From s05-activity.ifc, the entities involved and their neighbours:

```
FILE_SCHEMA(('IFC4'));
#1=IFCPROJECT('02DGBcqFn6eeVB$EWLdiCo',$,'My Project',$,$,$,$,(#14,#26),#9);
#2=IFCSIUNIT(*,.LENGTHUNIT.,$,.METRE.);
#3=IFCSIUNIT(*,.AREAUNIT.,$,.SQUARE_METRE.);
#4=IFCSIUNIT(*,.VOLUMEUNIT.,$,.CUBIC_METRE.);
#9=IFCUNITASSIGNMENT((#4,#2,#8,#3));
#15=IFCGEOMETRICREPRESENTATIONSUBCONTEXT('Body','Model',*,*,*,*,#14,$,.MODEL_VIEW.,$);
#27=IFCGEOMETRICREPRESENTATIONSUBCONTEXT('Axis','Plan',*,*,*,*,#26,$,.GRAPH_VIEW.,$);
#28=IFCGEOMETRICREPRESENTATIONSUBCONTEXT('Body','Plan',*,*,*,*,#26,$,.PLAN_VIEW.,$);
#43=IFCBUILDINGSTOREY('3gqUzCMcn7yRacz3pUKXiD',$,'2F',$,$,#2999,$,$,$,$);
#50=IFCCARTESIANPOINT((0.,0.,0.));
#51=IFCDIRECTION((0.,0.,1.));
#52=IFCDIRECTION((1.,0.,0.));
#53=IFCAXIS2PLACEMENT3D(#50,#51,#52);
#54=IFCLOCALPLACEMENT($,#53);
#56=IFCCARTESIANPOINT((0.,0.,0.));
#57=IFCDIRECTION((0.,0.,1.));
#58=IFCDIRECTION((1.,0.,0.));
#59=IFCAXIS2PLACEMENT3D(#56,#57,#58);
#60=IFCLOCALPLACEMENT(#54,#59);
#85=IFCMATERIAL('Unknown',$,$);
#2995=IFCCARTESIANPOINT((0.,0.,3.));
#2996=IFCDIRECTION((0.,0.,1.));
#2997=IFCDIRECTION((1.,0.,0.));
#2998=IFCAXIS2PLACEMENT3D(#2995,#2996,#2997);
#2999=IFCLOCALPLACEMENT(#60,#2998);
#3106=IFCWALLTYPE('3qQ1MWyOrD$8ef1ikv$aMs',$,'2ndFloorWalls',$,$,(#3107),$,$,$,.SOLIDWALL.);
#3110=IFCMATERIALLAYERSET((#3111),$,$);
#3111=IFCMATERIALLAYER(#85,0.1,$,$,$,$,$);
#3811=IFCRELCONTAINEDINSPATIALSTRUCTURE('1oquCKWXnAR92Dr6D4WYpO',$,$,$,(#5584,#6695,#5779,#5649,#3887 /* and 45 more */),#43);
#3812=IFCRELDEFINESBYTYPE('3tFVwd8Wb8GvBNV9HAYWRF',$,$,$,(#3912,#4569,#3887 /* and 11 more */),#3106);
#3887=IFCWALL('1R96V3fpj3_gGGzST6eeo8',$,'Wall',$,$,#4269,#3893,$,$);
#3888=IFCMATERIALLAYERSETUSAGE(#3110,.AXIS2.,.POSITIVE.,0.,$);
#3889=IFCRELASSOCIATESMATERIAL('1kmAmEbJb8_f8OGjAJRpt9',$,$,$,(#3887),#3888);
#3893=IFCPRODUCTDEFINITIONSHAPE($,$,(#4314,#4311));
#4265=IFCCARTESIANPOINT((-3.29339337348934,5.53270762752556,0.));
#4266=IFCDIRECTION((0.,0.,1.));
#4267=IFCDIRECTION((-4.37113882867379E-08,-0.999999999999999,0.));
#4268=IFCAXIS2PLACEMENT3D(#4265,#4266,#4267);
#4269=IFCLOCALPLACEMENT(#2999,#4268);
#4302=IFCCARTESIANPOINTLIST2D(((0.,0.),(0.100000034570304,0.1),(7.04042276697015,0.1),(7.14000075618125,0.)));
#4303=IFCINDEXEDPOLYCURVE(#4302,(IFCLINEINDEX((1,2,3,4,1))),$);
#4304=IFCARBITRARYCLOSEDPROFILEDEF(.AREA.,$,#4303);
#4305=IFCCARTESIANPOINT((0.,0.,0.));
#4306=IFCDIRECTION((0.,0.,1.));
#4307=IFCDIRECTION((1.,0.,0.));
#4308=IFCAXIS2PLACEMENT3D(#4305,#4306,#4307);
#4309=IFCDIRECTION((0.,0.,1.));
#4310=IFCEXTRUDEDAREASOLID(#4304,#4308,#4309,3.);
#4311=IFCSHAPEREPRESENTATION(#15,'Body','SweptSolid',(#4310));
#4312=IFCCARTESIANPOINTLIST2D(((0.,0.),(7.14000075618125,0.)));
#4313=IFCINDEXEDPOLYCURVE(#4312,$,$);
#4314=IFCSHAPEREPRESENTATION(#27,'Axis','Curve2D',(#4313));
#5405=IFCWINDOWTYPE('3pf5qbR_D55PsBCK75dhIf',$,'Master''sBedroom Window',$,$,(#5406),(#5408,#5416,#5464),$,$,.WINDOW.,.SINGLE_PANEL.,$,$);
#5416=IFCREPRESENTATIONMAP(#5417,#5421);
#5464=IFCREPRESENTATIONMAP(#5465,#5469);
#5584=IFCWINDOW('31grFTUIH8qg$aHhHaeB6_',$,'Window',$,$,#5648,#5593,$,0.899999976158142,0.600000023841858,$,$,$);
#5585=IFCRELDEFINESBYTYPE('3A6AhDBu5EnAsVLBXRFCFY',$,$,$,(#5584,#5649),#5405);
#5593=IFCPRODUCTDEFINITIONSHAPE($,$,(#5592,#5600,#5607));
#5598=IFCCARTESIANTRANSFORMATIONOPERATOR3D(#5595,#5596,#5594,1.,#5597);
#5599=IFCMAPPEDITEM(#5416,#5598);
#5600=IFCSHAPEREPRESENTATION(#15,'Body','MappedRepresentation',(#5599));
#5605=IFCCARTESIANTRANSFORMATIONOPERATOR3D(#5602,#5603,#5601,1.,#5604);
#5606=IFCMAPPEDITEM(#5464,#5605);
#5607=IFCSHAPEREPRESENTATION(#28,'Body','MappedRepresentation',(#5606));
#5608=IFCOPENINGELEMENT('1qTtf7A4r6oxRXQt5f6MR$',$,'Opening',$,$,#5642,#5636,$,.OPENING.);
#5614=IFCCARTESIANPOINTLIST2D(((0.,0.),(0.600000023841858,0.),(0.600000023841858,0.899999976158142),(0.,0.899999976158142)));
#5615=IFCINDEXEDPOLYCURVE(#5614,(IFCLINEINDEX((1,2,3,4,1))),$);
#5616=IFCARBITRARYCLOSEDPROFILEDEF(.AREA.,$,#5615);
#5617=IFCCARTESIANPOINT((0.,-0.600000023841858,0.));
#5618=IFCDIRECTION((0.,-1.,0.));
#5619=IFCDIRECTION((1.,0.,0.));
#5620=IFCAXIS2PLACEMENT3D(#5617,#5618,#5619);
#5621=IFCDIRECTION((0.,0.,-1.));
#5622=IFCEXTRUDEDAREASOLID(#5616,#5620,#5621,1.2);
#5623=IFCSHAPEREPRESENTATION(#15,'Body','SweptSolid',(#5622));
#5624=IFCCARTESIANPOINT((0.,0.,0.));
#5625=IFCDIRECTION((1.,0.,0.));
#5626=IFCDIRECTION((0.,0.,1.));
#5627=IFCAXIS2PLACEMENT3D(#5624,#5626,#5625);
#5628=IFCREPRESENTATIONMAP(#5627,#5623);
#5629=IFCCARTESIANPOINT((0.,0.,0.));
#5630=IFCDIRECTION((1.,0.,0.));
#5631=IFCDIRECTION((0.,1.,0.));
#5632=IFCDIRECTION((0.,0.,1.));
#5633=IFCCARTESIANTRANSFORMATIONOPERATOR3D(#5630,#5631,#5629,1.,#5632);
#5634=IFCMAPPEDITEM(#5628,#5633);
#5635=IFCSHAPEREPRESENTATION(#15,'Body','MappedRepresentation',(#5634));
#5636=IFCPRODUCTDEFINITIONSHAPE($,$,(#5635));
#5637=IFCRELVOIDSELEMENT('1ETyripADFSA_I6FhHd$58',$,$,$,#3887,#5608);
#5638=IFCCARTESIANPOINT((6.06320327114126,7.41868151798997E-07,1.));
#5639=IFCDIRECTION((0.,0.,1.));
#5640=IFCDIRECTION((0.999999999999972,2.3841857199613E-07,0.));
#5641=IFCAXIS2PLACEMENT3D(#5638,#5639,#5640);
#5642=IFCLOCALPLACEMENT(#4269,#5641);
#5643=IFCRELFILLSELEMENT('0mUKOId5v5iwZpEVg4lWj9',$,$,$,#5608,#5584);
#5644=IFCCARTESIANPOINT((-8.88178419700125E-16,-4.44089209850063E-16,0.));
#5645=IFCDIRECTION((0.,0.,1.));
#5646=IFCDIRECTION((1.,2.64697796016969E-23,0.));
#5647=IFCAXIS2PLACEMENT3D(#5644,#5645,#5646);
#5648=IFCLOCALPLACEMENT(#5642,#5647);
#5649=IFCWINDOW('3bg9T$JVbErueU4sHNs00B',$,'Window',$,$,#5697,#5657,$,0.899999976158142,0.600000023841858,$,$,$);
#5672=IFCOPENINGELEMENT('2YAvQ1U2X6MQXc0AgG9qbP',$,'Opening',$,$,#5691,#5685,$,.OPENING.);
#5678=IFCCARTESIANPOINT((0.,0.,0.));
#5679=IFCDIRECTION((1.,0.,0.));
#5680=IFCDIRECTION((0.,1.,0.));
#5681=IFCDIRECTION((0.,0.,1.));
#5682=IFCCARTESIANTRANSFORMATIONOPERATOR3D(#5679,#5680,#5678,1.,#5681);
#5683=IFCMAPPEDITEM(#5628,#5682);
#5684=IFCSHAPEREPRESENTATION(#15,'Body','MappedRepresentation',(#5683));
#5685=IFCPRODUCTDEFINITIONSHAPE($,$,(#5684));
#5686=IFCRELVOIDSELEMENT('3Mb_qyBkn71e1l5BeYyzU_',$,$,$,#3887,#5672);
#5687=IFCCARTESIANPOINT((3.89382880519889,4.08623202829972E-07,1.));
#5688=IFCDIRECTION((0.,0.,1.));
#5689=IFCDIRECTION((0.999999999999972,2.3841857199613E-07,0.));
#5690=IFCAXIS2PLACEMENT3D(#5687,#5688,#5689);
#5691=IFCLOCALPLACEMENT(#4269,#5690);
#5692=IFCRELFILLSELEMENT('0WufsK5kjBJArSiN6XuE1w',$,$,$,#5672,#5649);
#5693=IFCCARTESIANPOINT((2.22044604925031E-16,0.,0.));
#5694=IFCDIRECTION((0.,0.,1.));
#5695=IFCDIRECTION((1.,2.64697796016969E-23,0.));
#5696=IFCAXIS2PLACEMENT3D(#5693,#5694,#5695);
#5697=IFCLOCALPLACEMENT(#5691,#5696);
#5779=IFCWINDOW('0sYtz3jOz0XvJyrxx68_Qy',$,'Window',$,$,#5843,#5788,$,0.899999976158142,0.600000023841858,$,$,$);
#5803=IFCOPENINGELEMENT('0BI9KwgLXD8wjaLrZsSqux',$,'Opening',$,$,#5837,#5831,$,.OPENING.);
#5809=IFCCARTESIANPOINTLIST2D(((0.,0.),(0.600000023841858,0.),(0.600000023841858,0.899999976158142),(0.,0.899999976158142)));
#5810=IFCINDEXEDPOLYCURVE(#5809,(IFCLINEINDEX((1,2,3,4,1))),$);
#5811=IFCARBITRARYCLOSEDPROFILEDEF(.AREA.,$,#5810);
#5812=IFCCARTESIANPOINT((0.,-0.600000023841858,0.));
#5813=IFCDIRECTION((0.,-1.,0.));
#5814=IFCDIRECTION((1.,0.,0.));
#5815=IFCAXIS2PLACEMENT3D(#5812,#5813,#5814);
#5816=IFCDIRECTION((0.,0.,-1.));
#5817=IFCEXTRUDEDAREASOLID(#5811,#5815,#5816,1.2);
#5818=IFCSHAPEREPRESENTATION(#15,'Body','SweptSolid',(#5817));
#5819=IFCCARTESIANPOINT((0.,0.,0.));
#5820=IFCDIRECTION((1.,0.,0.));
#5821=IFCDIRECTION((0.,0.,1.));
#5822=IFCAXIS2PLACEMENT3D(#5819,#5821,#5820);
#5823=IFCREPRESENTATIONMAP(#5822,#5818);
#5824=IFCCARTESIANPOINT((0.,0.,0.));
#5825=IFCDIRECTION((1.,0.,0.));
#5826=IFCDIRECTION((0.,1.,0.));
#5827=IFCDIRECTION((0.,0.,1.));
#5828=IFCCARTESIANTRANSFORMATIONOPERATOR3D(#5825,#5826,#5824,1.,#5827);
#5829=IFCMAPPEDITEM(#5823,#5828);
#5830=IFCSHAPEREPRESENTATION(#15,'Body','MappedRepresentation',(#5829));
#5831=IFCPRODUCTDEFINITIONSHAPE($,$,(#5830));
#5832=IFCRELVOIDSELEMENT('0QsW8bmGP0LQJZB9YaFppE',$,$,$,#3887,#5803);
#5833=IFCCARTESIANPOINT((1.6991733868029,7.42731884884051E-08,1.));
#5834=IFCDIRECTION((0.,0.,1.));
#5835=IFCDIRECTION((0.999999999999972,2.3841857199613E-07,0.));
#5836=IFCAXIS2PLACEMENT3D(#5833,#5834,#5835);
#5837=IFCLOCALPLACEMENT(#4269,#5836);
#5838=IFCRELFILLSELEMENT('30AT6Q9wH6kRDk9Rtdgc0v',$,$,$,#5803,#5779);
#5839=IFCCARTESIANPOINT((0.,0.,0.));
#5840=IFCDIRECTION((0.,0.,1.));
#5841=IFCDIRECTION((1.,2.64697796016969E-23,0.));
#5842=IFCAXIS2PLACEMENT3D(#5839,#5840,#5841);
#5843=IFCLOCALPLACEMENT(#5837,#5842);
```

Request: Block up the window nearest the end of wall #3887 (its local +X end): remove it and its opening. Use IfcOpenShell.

```python
import ifcopenshell
import ifcopenshell.api.feature
import ifcopenshell.api.root
import ifcopenshell.geom
import ifcopenshell.util.shape

model = ifcopenshell.open("s05-activity.ifc")
settings = ifcopenshell.geom.settings()


def volume(element):
    """Net volume in cubic metres, openings subtracted."""
    shape = ifcopenshell.geom.create_shape(settings, element)
    return ifcopenshell.util.shape.get_volume(shape.geometry)


window = model.by_guid("31grFTUIH8qg$aHhHaeB6_")
opening = window.FillsVoids[0].RelatingOpeningElement
wall = opening.VoidsElements[0].RelatingBuildingElement
before = volume(wall)

ifcopenshell.api.root.remove_product(model, product=window)
ifcopenshell.api.feature.remove_feature(model, feature=opening)

after = volume(wall)

print(f"wall volume {before:.3f} -> {after:.3f} m3")

model.write("s05-activity_v2.ifc")
```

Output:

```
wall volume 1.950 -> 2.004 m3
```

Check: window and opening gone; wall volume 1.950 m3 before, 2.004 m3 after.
